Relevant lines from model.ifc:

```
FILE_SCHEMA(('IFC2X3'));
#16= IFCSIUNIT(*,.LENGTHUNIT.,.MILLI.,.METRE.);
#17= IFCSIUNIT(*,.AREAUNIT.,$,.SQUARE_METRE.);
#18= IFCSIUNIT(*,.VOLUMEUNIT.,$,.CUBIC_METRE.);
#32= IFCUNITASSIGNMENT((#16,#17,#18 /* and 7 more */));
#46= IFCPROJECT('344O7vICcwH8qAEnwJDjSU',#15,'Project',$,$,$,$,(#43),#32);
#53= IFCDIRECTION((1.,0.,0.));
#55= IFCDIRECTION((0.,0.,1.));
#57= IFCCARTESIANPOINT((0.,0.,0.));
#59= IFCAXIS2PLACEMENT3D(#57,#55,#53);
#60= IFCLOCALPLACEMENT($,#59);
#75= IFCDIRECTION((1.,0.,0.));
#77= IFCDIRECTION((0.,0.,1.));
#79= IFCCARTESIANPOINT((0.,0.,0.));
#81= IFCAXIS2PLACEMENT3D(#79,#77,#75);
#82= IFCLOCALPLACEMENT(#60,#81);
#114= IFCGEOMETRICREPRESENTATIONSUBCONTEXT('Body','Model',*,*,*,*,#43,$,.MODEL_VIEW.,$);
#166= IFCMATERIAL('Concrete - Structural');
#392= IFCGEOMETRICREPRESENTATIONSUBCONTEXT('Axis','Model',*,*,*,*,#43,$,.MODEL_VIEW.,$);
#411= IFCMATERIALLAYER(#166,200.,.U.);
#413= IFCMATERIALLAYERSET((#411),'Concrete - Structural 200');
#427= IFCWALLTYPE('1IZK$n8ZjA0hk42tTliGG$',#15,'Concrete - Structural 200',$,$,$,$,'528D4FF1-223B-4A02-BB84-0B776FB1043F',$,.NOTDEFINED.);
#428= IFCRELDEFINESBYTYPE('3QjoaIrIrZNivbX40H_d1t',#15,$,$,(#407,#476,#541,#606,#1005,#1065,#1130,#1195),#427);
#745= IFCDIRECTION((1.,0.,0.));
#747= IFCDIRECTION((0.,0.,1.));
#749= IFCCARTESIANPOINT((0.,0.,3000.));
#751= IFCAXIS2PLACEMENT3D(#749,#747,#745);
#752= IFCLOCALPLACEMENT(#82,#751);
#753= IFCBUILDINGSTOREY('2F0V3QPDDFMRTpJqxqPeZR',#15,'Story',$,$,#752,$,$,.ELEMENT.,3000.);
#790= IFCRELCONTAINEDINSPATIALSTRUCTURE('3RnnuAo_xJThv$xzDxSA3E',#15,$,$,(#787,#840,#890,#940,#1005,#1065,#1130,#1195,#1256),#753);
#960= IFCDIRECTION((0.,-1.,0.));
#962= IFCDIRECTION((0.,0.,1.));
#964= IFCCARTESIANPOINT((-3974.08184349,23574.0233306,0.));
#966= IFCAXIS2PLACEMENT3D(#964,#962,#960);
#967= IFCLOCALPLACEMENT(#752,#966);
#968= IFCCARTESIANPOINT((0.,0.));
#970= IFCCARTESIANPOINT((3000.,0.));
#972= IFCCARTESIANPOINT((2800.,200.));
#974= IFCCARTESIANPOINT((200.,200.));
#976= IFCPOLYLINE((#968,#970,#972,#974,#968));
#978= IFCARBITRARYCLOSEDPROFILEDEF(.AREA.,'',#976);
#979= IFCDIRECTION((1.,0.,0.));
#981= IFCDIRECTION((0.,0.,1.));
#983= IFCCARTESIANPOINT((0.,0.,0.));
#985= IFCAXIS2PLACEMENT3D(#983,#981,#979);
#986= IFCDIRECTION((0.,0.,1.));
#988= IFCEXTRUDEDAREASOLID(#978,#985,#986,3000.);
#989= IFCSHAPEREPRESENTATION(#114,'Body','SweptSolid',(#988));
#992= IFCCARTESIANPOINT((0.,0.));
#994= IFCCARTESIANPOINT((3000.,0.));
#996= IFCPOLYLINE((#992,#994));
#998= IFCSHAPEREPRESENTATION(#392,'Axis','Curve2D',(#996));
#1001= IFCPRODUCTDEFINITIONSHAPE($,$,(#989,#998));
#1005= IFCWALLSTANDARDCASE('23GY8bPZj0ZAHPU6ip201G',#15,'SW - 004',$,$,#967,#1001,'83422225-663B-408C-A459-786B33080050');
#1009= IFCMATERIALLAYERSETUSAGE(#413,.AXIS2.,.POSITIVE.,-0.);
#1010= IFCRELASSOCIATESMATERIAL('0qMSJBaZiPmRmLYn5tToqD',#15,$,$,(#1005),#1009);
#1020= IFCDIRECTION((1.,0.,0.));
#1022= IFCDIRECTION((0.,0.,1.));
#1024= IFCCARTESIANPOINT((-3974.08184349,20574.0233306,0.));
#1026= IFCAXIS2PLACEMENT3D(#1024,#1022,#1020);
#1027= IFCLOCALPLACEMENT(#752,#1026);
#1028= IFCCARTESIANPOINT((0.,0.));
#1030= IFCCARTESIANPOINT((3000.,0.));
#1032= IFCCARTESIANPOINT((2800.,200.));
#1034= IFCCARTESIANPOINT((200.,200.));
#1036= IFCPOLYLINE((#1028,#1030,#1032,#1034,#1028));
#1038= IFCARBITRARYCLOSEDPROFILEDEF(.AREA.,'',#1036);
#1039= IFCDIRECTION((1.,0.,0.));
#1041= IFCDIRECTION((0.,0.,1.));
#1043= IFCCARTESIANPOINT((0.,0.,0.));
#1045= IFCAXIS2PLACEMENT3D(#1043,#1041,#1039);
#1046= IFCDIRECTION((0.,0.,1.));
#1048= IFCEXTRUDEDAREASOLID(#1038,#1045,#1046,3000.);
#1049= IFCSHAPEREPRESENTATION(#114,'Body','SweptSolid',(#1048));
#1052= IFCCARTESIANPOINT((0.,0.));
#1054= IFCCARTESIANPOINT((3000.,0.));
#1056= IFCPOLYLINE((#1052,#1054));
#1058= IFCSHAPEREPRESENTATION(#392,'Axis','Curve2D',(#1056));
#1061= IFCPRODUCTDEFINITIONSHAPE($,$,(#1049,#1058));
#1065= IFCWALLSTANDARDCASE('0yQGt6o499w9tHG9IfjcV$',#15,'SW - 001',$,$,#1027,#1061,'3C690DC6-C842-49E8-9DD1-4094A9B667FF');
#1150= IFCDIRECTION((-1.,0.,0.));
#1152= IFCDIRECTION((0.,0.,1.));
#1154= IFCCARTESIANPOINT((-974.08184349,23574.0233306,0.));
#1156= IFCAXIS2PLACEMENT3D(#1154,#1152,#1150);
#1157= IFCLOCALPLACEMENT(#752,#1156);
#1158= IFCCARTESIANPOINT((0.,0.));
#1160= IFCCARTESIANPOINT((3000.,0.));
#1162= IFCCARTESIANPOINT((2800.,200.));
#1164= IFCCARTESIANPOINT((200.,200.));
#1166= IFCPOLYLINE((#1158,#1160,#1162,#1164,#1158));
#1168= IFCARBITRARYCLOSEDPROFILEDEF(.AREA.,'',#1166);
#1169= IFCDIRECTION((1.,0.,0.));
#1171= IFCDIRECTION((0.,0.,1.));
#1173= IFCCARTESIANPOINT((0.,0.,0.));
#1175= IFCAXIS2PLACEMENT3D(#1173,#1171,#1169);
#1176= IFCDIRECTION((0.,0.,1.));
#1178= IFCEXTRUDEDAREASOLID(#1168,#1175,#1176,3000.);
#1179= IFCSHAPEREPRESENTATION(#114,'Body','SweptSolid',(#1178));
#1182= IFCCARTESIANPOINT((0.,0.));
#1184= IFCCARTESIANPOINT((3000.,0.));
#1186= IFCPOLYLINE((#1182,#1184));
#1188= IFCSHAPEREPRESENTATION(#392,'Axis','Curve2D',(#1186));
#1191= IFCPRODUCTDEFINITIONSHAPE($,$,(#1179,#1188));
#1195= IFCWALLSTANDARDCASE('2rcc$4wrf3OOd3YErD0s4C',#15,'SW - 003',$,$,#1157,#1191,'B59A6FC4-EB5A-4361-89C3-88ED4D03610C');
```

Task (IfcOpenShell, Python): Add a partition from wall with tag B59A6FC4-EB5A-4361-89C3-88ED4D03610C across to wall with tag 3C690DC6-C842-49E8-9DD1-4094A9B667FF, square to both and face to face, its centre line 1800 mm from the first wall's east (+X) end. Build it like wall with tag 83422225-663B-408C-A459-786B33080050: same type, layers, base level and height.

```python
import numpy as np
import ifcopenshell
import ifcopenshell.api.geometry
import ifcopenshell.api.material
import ifcopenshell.api.pset
import ifcopenshell.api.root
import ifcopenshell.api.spatial
import ifcopenshell.api.type
import ifcopenshell.geom
import ifcopenshell.util.element
import ifcopenshell.util.placement
import ifcopenshell.util.representation
import ifcopenshell.util.shape
import ifcopenshell.util.unit

model = ifcopenshell.open("model.ifc")
unit_scale = ifcopenshell.util.unit.calculate_unit_scale(model)
settings = ifcopenshell.geom.settings()
settings.set("use-world-coords", True)

start_wall = model.by_guid("2rcc$4wrf3OOd3YErD0s4C")
end_wall = model.by_guid("0yQGt6o499w9tHG9IfjcV$")
like = model.by_id(1005)
matrix = ifcopenshell.util.placement.get_local_placement(start_wall.ObjectPlacement)
matrix[:3, 3] *= unit_scale


def extent(element):
    """Bounding box in the first wall's axes, in metres."""
    shape = ifcopenshell.geom.create_shape(settings, element)
    points = (ifcopenshell.util.shape.get_vertices(shape.geometry) - matrix[:3, 3]) @ matrix[:3, :3]
    return points.min(axis=0), points.max(axis=0)


y_start = extent(start_wall)[1][1]
y_end = extent(end_wall)[0][1]
like_min, like_max = extent(like)
length, height = float(abs(y_end - y_start)), float(like_max[2] - like_min[2])
layer_set = ifcopenshell.util.element.get_material(like, should_skip_usage=True)
thickness = sum(layer.LayerThickness for layer in layer_set.MaterialLayers) * unit_scale

wall = ifcopenshell.api.root.create_entity(model, ifc_class="IfcWallStandardCase", name="New partition")
storey = ifcopenshell.util.element.get_container(like)
ifcopenshell.api.spatial.assign_container(model, products=[wall], relating_structure=storey)
ifcopenshell.api.type.assign_type(
    model, related_objects=[wall], relating_type=ifcopenshell.util.element.get_type(like), should_map_representations=False
)
rel = ifcopenshell.api.material.assign_material(
    model, products=[wall], type="IfcMaterialLayerSetUsage", material=layer_set
)
rel.RelatingMaterial.OffsetFromReferenceLine = -thickness / 2 / unit_scale
pset = ifcopenshell.api.pset.add_pset(model, product=wall, name="Pset_WallCommon")
ifcopenshell.api.pset.edit_pset(model, pset=pset, properties={"IsExternal": False, "LoadBearing": False})

# The axis runs down the middle of the wall.
axis = ifcopenshell.api.geometry.add_axis_representation(
    model, context=ifcopenshell.util.representation.get_context(model, "Model", "Axis"), axis=[(0.0, 0.0), (length, 0.0)]
)
body = ifcopenshell.api.geometry.add_wall_representation(
    model,
    context=ifcopenshell.util.representation.get_context(model, "Model", "Body", "MODEL_VIEW"),
    length=length,
    height=height,
    thickness=thickness,
    offset=-thickness / 2,
)
for representation in (axis, body):
    ifcopenshell.api.geometry.assign_representation(model, product=wall, representation=representation)

placement = matrix @ ifcopenshell.util.placement.rotation(90, "Z")
placement[:, 3] = matrix @ np.array([extent(start_wall)[0][0] + 1.8, y_start, like_min[2], 1.0])
ifcopenshell.api.geometry.edit_object_placement(model, product=wall, matrix=placement)

print(f"partition {length:.3f} m long, {height:.3f} m high, {thickness:.3f} m thick")

model.write("model-out.ifc")
```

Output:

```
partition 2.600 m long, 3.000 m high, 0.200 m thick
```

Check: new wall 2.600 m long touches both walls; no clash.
